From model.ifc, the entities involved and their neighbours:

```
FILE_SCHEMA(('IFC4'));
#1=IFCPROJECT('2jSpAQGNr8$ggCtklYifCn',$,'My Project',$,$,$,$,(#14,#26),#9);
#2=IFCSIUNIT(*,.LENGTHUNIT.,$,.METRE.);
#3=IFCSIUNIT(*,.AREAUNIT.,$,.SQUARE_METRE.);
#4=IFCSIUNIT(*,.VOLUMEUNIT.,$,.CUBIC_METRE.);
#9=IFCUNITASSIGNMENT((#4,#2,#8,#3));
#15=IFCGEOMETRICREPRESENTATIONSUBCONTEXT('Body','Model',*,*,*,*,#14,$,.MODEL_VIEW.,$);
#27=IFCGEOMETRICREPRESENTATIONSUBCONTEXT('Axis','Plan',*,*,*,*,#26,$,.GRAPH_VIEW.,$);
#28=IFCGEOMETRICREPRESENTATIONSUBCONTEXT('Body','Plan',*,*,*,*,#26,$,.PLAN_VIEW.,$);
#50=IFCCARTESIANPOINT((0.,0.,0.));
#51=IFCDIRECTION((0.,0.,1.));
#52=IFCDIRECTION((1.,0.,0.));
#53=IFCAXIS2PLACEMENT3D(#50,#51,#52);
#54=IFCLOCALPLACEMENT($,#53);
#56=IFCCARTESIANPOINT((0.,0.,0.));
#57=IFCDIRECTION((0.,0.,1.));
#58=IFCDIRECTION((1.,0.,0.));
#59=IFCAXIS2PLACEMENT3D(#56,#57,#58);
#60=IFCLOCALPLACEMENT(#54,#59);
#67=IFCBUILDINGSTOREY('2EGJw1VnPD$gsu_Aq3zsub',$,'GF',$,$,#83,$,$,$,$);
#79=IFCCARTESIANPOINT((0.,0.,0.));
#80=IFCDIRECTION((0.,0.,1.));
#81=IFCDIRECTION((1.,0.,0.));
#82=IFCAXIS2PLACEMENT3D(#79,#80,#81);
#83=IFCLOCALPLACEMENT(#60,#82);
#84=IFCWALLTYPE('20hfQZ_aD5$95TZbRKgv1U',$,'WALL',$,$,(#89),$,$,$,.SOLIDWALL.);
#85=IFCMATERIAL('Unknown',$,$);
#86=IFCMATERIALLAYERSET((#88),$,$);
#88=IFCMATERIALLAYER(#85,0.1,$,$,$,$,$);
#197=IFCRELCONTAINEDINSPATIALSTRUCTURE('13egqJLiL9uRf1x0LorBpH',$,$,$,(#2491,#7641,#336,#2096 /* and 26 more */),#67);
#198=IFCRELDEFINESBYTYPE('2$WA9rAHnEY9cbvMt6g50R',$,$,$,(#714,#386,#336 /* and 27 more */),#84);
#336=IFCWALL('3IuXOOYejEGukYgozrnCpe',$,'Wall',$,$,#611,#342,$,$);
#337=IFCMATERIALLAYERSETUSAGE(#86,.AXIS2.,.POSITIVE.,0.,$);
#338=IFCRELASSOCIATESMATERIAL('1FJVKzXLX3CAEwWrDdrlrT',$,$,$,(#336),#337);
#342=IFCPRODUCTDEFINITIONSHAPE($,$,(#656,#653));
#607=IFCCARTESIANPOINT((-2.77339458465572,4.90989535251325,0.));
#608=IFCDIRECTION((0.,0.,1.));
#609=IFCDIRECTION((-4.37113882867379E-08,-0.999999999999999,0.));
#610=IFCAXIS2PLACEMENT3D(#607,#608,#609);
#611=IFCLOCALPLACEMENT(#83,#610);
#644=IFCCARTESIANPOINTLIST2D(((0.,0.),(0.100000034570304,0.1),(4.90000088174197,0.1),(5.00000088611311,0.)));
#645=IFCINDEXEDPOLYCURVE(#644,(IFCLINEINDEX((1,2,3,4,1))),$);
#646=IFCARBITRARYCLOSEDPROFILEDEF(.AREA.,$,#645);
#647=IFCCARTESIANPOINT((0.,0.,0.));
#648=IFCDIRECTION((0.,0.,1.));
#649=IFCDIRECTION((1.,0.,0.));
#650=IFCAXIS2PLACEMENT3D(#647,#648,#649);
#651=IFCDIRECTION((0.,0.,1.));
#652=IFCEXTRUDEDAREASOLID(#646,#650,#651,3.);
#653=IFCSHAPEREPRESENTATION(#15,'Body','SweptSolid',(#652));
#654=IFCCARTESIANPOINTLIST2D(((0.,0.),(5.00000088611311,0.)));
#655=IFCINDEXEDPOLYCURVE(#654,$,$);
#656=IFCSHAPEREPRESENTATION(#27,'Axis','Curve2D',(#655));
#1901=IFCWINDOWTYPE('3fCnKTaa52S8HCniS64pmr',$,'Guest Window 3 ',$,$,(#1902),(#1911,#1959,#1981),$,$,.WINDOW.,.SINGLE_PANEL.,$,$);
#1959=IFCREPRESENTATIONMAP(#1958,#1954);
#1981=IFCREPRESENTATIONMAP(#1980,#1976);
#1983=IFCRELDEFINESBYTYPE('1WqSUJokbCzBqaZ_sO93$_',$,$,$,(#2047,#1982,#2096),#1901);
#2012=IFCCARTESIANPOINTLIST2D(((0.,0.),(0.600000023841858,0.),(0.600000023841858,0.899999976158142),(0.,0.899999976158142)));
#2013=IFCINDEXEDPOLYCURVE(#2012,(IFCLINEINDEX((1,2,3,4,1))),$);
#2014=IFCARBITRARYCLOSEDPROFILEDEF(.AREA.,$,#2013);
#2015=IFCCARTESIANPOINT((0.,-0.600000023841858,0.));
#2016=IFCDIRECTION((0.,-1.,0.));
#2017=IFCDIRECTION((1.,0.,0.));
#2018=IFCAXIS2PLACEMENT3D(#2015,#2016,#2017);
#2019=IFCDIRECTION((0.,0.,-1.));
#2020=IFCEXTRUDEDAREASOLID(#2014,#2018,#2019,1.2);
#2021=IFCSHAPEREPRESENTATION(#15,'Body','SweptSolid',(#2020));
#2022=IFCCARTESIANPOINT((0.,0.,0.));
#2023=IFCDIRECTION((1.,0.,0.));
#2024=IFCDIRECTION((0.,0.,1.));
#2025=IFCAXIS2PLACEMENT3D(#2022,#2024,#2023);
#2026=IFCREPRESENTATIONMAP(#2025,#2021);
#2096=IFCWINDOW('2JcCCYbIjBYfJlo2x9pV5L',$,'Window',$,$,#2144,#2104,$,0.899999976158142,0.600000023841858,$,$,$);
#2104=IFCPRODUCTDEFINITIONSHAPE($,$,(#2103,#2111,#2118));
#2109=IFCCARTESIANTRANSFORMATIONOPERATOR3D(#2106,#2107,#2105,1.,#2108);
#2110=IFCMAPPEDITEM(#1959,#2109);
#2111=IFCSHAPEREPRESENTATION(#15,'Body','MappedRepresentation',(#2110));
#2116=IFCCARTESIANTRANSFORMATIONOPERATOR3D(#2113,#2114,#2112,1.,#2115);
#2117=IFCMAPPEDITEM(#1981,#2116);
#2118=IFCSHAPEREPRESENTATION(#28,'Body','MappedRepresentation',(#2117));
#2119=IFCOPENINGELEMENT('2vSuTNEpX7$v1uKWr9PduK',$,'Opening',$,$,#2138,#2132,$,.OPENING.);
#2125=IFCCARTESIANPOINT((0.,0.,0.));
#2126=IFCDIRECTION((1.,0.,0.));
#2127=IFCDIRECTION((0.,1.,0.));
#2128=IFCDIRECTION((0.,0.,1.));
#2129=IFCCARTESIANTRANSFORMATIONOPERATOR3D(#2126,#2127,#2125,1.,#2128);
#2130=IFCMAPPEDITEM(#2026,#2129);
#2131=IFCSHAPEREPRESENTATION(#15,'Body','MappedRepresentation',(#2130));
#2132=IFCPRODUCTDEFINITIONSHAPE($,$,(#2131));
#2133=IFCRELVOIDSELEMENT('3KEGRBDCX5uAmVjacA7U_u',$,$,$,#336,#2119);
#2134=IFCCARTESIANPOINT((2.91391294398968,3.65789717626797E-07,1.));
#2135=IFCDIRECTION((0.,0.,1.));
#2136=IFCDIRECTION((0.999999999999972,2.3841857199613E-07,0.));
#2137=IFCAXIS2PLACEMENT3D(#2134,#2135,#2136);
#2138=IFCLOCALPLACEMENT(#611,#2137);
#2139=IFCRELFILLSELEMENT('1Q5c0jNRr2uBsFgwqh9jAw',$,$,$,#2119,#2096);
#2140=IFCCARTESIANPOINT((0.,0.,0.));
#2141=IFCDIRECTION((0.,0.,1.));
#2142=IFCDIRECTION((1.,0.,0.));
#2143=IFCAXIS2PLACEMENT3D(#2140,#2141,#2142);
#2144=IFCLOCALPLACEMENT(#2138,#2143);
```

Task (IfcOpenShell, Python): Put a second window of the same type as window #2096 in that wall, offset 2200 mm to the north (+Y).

```python
import ifcopenshell
import ifcopenshell.api.feature
import ifcopenshell.api.geometry
import ifcopenshell.api.root
import ifcopenshell.geom
import ifcopenshell.util.element
import ifcopenshell.util.placement
import ifcopenshell.util.shape
import ifcopenshell.util.unit

model = ifcopenshell.open("model.ifc")
unit_scale = ifcopenshell.util.unit.calculate_unit_scale(model)
settings = ifcopenshell.geom.settings()


def volume(element):
    """Net volume in cubic metres, openings subtracted."""
    shape = ifcopenshell.geom.create_shape(settings, element)
    return ifcopenshell.util.shape.get_volume(shape.geometry)


window = model.by_guid("2JcCCYbIjBYfJlo2x9pV5L")
opening = window.FillsVoids[0].RelatingOpeningElement
wall = opening.VoidsElements[0].RelatingBuildingElement
before = volume(wall)
shift = ifcopenshell.util.placement.get_local_placement(wall.ObjectPlacement)[:3, 0] * -2.2 / unit_scale

# copy_class copies the void relationship, type, container and properties, but no geometry.
new_opening = ifcopenshell.api.root.copy_class(model, product=opening)
new_opening.Representation = ifcopenshell.util.element.copy_deep(
    model, opening.Representation, exclude=["IfcGeometricRepresentationContext", "IfcRepresentationMap"]
)
new_window = ifcopenshell.api.root.copy_class(model, product=window)
new_window.Representation = ifcopenshell.util.element.copy_deep(
    model, window.Representation, exclude=["IfcGeometricRepresentationContext", "IfcRepresentationMap"]
)
ifcopenshell.api.feature.add_filling(model, opening=new_opening, element=new_window)

for old, new in ((opening, new_opening), (window, new_window)):
    matrix = ifcopenshell.util.placement.get_local_placement(old.ObjectPlacement)
    matrix[:3, 3] += shift
    ifcopenshell.api.geometry.edit_object_placement(model, product=new, matrix=matrix, is_si=False)

after = volume(wall)

print(f"wall volume {before:.3f} -> {after:.3f} m3")

model.write("model_rev.ifc")
```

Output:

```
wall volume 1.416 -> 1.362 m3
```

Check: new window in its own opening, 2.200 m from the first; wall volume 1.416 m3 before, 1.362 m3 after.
